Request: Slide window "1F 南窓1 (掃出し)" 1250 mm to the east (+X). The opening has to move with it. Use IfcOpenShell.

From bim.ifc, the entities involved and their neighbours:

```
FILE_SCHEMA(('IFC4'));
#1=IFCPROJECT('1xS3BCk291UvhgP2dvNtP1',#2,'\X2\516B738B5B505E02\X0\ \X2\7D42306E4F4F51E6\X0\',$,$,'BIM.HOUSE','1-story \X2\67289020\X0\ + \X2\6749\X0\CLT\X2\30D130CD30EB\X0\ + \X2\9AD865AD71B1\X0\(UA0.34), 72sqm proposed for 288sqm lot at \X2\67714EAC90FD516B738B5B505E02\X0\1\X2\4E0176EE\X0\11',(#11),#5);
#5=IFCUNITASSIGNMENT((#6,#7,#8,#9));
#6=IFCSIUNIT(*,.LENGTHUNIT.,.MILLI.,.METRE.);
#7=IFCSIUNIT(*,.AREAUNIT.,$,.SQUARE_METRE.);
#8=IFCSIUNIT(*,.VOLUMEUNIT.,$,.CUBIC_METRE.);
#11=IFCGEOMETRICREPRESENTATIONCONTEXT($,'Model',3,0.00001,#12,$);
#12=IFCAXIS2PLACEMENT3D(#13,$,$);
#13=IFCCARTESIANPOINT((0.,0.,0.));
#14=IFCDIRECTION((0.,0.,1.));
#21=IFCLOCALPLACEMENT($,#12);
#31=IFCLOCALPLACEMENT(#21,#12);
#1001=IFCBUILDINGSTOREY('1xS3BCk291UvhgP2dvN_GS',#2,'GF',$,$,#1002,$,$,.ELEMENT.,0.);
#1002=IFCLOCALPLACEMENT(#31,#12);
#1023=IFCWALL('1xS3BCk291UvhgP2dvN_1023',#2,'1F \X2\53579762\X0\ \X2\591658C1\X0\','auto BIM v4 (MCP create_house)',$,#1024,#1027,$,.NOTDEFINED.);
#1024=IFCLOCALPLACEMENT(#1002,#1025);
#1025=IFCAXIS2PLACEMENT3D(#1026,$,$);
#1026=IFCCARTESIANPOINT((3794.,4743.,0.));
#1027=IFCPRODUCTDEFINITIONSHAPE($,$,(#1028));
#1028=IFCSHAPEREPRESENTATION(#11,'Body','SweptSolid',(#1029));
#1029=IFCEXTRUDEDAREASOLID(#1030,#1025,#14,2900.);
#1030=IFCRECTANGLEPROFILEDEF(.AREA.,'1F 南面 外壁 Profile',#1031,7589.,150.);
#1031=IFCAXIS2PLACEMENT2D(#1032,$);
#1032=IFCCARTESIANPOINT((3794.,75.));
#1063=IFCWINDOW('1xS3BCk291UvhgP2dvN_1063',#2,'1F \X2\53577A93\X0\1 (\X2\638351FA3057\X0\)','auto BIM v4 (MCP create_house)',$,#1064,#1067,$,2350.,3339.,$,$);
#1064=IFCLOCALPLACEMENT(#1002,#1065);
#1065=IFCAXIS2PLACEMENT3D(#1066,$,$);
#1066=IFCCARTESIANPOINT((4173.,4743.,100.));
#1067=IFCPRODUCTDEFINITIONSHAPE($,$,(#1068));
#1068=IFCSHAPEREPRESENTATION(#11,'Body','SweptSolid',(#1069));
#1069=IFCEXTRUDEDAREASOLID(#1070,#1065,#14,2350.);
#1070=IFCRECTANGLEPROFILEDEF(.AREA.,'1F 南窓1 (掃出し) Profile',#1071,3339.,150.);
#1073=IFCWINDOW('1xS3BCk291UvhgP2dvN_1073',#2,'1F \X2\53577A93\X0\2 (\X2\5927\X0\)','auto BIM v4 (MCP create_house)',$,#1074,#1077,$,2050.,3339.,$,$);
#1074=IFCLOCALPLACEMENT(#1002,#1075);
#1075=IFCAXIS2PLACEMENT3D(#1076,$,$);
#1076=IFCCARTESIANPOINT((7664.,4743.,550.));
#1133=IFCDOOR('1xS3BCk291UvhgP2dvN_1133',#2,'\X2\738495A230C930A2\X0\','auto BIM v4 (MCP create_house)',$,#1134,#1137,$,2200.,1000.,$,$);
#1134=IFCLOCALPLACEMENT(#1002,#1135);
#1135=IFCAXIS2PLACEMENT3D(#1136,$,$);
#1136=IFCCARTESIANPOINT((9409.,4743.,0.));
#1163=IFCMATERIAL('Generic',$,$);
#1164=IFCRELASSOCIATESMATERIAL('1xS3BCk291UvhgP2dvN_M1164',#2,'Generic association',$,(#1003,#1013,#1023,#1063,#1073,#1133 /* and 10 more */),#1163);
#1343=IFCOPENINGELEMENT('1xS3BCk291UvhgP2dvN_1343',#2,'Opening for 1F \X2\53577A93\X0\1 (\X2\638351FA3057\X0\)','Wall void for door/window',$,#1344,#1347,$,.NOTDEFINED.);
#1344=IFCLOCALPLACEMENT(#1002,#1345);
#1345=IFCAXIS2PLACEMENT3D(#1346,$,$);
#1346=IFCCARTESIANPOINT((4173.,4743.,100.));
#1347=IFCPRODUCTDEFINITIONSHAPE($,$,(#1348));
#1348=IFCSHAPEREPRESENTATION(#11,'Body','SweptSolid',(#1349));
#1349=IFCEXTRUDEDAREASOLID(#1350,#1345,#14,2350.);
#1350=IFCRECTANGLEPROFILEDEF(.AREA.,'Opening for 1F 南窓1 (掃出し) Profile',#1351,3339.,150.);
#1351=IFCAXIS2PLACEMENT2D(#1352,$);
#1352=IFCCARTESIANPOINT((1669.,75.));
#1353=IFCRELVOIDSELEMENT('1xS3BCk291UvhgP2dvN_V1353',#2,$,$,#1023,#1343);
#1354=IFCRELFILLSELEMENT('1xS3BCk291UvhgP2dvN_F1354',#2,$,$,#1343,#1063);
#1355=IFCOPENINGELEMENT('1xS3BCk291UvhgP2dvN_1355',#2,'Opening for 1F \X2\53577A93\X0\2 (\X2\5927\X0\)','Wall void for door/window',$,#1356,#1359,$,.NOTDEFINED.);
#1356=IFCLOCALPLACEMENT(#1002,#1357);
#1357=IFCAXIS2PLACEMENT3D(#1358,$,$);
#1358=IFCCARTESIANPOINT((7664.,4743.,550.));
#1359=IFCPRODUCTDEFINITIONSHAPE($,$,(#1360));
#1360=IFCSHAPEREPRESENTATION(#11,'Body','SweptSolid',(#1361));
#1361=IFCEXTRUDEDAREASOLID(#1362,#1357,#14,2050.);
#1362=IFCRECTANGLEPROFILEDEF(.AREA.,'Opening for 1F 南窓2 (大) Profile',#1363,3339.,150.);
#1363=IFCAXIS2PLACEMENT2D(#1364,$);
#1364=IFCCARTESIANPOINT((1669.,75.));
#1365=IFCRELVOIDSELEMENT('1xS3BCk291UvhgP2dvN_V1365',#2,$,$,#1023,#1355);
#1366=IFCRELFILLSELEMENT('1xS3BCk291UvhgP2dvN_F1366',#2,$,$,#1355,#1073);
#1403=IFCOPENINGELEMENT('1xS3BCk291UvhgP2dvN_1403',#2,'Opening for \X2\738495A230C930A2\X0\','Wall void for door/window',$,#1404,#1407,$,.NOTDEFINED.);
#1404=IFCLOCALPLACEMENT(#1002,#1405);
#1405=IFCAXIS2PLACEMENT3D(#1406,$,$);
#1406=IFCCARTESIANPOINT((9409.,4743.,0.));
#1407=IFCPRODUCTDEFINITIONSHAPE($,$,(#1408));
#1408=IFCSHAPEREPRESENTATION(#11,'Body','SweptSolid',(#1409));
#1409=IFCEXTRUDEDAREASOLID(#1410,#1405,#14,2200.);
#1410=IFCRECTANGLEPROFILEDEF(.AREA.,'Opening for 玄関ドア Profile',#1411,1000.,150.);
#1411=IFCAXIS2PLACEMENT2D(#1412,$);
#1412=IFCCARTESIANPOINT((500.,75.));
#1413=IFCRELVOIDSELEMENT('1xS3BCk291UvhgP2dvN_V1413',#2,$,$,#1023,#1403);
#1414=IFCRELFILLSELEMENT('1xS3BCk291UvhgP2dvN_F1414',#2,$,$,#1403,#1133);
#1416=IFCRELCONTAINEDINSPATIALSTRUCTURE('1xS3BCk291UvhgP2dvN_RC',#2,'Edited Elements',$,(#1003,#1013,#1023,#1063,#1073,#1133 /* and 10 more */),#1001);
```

```python
import ifcopenshell
import ifcopenshell.api.geometry
import ifcopenshell.util.placement
import ifcopenshell.util.unit

model = ifcopenshell.open("bim.ifc")
unit_scale = ifcopenshell.util.unit.calculate_unit_scale(model)

window = model.by_guid("1xS3BCk291UvhgP2dvN_1063")
opening = window.FillsVoids[0].RelatingOpeningElement
wall = opening.VoidsElements[0].RelatingBuildingElement

wall_matrix = ifcopenshell.util.placement.get_local_placement(wall.ObjectPlacement)
shift = wall_matrix[:3, 0] * 1.25 / unit_scale
before = ifcopenshell.util.placement.get_local_placement(window.ObjectPlacement)[:3, 3].copy()

# The window is not placed relative to its opening, so move both.
for product in (opening, window):
    matrix = ifcopenshell.util.placement.get_local_placement(product.ObjectPlacement)
    matrix[:3, 3] += shift
    ifcopenshell.api.geometry.edit_object_placement(model, product=product, matrix=matrix, is_si=False)

after = ifcopenshell.util.placement.get_local_placement(window.ObjectPlacement)[:3, 3]
print("window moved by", (after - before).round(3) + 0.0)

model.write("bim_v2.ifc")
```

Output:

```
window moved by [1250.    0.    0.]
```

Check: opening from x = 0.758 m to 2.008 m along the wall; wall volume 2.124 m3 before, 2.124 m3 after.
